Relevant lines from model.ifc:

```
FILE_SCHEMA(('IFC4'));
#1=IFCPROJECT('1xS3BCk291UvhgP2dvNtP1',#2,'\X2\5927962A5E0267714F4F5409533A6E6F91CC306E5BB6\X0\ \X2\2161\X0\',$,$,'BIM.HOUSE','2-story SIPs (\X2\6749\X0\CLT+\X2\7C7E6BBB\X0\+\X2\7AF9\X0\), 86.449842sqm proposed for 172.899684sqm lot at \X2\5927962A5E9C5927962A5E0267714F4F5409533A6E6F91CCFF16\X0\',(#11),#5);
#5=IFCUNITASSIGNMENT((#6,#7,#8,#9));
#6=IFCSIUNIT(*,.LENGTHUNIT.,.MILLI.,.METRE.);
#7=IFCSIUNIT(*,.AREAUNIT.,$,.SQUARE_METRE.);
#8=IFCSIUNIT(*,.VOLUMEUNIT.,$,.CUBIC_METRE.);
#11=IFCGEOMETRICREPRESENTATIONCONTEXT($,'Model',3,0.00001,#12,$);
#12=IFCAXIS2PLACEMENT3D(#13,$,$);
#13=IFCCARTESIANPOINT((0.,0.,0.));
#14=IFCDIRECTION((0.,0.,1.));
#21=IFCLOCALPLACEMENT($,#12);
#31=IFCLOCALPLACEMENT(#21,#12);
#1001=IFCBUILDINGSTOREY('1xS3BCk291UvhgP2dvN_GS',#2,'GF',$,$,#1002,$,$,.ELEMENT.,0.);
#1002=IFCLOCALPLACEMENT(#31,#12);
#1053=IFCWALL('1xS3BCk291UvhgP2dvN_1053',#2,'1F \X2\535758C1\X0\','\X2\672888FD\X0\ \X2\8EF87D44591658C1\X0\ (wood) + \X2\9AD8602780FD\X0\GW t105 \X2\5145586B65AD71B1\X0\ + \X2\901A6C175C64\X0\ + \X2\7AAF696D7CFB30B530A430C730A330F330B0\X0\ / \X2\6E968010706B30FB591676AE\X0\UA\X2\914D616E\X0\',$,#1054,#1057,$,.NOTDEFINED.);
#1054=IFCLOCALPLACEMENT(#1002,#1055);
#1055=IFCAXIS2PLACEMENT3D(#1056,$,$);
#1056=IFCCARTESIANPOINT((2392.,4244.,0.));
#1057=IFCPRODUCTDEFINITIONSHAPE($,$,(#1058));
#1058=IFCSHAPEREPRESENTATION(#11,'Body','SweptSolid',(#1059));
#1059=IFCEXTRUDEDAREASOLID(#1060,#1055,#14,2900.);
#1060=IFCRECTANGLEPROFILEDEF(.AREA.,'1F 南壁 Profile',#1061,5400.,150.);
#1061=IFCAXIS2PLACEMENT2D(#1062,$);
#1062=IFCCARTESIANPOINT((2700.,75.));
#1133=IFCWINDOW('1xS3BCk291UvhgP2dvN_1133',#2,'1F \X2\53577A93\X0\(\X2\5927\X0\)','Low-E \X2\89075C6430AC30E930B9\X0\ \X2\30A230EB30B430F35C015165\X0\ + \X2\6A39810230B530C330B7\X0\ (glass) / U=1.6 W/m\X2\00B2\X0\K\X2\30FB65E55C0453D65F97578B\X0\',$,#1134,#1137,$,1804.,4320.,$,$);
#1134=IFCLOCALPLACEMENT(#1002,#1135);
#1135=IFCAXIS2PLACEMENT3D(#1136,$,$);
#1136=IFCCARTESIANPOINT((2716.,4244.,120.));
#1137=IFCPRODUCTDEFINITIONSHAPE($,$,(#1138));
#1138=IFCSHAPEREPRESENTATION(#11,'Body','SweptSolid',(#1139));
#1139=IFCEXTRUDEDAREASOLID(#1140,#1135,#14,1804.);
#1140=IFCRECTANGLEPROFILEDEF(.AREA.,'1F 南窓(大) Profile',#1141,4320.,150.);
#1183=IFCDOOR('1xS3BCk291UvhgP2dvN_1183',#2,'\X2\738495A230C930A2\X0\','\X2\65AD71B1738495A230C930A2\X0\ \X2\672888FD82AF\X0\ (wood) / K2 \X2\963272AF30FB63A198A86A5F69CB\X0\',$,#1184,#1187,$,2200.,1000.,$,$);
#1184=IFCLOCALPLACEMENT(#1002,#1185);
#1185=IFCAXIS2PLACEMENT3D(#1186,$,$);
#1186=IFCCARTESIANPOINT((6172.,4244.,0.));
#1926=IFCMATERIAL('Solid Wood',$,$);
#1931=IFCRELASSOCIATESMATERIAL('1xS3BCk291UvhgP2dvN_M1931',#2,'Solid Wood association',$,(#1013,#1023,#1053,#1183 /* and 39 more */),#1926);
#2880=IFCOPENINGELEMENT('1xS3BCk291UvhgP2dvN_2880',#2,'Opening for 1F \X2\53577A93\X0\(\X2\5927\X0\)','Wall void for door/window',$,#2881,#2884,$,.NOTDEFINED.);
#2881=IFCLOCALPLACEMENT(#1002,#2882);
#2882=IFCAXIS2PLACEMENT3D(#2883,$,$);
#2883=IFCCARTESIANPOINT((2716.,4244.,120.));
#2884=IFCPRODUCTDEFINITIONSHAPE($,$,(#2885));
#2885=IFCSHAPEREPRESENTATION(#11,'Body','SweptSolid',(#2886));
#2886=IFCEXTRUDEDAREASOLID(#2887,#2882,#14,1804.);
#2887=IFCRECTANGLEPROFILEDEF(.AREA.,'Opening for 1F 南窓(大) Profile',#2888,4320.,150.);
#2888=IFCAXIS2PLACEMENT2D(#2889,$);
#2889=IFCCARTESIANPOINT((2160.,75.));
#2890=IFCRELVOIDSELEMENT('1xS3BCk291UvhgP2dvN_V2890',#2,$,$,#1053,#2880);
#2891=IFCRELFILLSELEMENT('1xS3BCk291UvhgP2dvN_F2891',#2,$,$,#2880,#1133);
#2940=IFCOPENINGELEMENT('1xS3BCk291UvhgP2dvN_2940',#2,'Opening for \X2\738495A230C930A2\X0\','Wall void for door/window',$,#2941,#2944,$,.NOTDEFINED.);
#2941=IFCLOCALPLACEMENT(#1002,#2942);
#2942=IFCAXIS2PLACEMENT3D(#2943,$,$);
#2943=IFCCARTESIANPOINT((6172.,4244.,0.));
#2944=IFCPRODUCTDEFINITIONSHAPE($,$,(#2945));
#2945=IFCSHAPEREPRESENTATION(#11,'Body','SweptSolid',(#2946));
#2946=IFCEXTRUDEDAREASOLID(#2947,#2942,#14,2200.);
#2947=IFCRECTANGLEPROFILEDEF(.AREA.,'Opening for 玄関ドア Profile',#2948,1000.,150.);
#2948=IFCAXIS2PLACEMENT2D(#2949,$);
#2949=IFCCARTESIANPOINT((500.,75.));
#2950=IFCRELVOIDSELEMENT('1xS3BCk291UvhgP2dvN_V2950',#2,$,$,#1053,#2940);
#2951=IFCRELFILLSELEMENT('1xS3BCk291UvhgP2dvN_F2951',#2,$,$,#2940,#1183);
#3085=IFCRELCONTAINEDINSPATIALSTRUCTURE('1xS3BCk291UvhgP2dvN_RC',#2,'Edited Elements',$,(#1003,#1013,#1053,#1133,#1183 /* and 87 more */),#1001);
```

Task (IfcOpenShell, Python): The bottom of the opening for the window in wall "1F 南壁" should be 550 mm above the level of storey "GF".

```python
import numpy as np
import ifcopenshell
import ifcopenshell.api.geometry
import ifcopenshell.geom
import ifcopenshell.util.element
import ifcopenshell.util.placement
import ifcopenshell.util.shape
import ifcopenshell.util.unit

model = ifcopenshell.open("model.ifc")
unit_scale = ifcopenshell.util.unit.calculate_unit_scale(model)

window = model.by_guid("1xS3BCk291UvhgP2dvN_1133")
opening = window.FillsVoids[0].RelatingOpeningElement
storey = ifcopenshell.util.element.get_container(window, ifc_class="IfcBuildingStorey")
level = ifcopenshell.util.placement.get_local_placement(storey.ObjectPlacement)[2, 3]

# The opening's origin need not be at the sill, so measure its lowest point.
shape = ifcopenshell.geom.create_shape(ifcopenshell.geom.settings(), opening)
bottom = ifcopenshell.util.shape.get_shape_bottom_elevation(shape, shape.geometry) / unit_scale
dz = level + 0.55 / unit_scale - bottom

shift = np.array([0.0, 0.0, dz])
# The window is not placed relative to its opening, so move both.
for product in (opening, window):
    matrix = ifcopenshell.util.placement.get_local_placement(product.ObjectPlacement)
    matrix[:3, 3] += shift
    ifcopenshell.api.geometry.edit_object_placement(model, product=product, matrix=matrix, is_si=False)

print(f"moved by {dz * unit_scale:+.3f} m")

model.write("model_v2.ifc")
```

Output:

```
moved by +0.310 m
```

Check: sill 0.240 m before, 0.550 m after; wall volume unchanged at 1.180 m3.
